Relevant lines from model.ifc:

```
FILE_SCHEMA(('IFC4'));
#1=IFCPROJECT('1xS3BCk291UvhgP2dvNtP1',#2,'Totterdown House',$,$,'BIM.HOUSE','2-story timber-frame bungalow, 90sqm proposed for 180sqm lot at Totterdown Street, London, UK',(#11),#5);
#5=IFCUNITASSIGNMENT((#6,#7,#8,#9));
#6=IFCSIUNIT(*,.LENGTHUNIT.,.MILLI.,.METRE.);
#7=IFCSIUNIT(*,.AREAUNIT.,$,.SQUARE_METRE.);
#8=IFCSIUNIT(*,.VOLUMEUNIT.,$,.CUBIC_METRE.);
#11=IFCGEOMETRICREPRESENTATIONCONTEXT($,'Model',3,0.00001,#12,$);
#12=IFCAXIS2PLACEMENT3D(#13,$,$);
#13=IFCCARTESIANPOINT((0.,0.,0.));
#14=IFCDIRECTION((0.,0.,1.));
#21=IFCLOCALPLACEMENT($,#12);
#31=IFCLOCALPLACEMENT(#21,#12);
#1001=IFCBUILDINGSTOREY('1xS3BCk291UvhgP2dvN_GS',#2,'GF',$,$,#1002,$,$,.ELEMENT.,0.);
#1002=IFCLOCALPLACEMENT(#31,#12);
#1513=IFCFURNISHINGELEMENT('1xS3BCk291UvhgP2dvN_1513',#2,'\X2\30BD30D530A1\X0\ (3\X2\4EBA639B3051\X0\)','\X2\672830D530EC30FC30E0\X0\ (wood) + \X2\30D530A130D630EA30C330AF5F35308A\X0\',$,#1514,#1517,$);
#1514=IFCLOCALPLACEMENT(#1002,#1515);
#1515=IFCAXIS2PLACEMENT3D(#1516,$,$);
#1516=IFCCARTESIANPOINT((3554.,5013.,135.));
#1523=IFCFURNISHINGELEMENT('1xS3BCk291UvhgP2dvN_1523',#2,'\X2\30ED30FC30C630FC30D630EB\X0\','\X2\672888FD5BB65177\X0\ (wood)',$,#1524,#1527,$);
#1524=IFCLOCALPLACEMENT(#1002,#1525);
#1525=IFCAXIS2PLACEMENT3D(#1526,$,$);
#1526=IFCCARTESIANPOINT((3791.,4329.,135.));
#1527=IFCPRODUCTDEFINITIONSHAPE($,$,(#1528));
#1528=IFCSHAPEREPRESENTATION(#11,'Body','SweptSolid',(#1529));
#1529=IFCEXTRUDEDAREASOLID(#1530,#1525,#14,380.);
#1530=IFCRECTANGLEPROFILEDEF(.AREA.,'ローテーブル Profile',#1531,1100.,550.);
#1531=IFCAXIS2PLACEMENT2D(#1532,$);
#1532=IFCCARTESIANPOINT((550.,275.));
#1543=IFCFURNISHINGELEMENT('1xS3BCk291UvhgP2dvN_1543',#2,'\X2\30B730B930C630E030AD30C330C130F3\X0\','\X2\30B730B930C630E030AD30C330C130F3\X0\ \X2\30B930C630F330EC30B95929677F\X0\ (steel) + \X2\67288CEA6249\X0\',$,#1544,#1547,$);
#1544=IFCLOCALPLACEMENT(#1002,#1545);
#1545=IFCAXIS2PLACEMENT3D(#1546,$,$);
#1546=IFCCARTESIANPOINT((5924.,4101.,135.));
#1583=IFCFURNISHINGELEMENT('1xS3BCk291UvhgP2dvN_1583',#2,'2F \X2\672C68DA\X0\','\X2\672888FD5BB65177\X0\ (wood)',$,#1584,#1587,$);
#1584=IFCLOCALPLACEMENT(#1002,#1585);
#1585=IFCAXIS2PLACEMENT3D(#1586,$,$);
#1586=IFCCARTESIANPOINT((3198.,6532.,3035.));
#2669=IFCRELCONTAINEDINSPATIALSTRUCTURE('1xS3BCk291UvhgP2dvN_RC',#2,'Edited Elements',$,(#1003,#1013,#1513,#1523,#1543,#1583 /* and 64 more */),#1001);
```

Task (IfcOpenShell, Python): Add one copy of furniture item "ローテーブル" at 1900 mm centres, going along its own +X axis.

```python
import ifcopenshell
import ifcopenshell.api.geometry
import ifcopenshell.api.root
import ifcopenshell.util.element
import ifcopenshell.util.placement
import ifcopenshell.util.unit

model = ifcopenshell.open("model.ifc")
unit_scale = ifcopenshell.util.unit.calculate_unit_scale(model)


def reuse_history(source, copy):
    """copy_class also copies each property set's owner history, people and application; keep the originals."""
    for rel in copy.IsDefinedBy:
        if rel.is_a("IfcRelDefinesByProperties") and (history := rel.RelatingPropertyDefinition.OwnerHistory):
            rel.RelatingPropertyDefinition.OwnerHistory = source.OwnerHistory
            ifcopenshell.util.element.remove_deep2(model, history)


source = model.by_guid("1xS3BCk291UvhgP2dvN_1523")
base = ifcopenshell.util.placement.get_local_placement(source.ObjectPlacement)
step = base[:3, 0] * 1.9 / unit_scale

for i in range(1, 2):
    copy = ifcopenshell.api.root.copy_class(model, product=source)
    copy.Representation = ifcopenshell.util.element.copy_deep(
        model, source.Representation, exclude=["IfcGeometricRepresentationContext", "IfcRepresentationMap"]
    )
    reuse_history(source, copy)
    matrix = base.copy()
    matrix[:3, 3] += i * step
    print("added at", matrix[:3, 3].round(3) + 0.0)
    ifcopenshell.api.geometry.edit_object_placement(model, product=copy, matrix=matrix, is_si=False)

model.write("model_updated.ifc")
```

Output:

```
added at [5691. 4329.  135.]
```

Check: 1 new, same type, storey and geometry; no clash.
